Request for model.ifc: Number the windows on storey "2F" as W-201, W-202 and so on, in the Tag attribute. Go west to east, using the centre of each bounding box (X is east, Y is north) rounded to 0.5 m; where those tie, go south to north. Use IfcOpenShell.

First a look at what the model holds.

```python
import ifcopenshell
import ifcopenshell.util.element
import ifcopenshell.util.placement

model = ifcopenshell.open("model.ifc")
print(model.schema)
storey = next(s for s in model.by_type("IfcBuildingStorey") if s.Name == "2F")
windows = [e for e in ifcopenshell.util.element.get_decomposition(storey) if e.is_a("IfcWindow")]
for e in sorted(windows, key=lambda e: e.id()):
    origin = ifcopenshell.util.placement.get_local_placement(e.ObjectPlacement)[:3, 3]
    print(e.id(), e.Tag, e.Name, origin.round(2) + 0.0, sep=" | ")
```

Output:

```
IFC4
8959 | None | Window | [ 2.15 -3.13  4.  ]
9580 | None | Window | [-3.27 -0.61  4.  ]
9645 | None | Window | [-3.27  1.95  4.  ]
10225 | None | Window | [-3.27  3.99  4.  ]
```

```python
import ifcopenshell
import ifcopenshell.geom
import ifcopenshell.util.element
import ifcopenshell.util.shape

model = ifcopenshell.open("model.ifc")
settings = ifcopenshell.geom.settings()
settings.set("use-world-coords", True)


def centre(element):
    shape = ifcopenshell.geom.create_shape(settings, element)
    return ifcopenshell.util.shape.get_bbox_centroid(shape.geometry)


storey = next(s for s in model.by_type("IfcBuildingStorey") if s.Name == "2F")
windows = [e for e in ifcopenshell.util.element.get_decomposition(storey) if e.is_a("IfcWindow")]

# Insertion points can sit at a corner or the storey origin, so sort by the geometry (in metres).
centres = {e: centre(e) for e in windows}
windows.sort(key=lambda e: (round(centres[e][0] / 0.5), centres[e][1]))

for i, e in enumerate(windows, start=1):
    number = f"W-2{i:02d}"
    e.Tag = number
    print(e.id(), number)

model.write("model_edited.ifc")
```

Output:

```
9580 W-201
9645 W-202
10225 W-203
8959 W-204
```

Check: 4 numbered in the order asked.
